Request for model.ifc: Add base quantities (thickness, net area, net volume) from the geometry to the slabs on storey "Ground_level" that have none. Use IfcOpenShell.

First a look at what the model holds.

```python
import ifcopenshell
import ifcopenshell.util.element
import ifcopenshell.util.unit

model = ifcopenshell.open("model.ifc")
print(model.schema)
for unit_type in ("LENGTHUNIT", "AREAUNIT", "VOLUMEUNIT"):
    print(unit_type, ifcopenshell.util.unit.calculate_unit_scale(model, unit_type))
storey = next(s for s in model.by_type("IfcBuildingStorey") if s.Name == "Ground_level")
slabs = [e for e in ifcopenshell.util.element.get_decomposition(storey) if e.is_a("IfcSlab")]
for e in sorted(slabs, key=lambda e: e.id()):
    print(e.id(), e.is_a(), e.Name, list(ifcopenshell.util.element.get_psets(e, qtos_only=True)), sep=" | ")
```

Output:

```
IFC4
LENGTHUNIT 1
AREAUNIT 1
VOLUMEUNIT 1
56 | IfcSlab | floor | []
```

```python
import ifcopenshell
import ifcopenshell.api.pset
import ifcopenshell.geom
import ifcopenshell.util.element
import ifcopenshell.util.shape
import ifcopenshell.util.unit

model = ifcopenshell.open("model.ifc")
unit_scale = ifcopenshell.util.unit.calculate_unit_scale(model)
area_scale = ifcopenshell.util.unit.calculate_unit_scale(model, "AREAUNIT")
volume_scale = ifcopenshell.util.unit.calculate_unit_scale(model, "VOLUMEUNIT")
settings = ifcopenshell.geom.settings()

storey = next(s for s in model.by_type("IfcBuildingStorey") if s.Name == "Ground_level")
slabs = [e for e in ifcopenshell.util.element.get_decomposition(storey) if e.is_a("IfcSlab")]

for e in sorted(slabs, key=lambda e: e.id()):
    if ifcopenshell.util.element.get_psets(e, qtos_only=True, should_inherit=False):
        continue
    # Geometry comes back in metres, in the element's own axes.
    shape = ifcopenshell.geom.create_shape(settings, e)
    values = {
        "Width": ifcopenshell.util.shape.get_z(shape.geometry) / unit_scale,
        "NetArea": ifcopenshell.util.shape.get_footprint_area(shape.geometry) / area_scale,
        "NetVolume": ifcopenshell.util.shape.get_volume(shape.geometry) / volume_scale,
    }
    qto = ifcopenshell.api.pset.add_qto(model, product=e, name="Qto_SlabBaseQuantities")
    ifcopenshell.api.pset.edit_qto(model, qto=qto, properties=values)
    print(e.id(), {k: round(v, 3) for k, v in values.items()})

model.write("model_rev.ifc")
```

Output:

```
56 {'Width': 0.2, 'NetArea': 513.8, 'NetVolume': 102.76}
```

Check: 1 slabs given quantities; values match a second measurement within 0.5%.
